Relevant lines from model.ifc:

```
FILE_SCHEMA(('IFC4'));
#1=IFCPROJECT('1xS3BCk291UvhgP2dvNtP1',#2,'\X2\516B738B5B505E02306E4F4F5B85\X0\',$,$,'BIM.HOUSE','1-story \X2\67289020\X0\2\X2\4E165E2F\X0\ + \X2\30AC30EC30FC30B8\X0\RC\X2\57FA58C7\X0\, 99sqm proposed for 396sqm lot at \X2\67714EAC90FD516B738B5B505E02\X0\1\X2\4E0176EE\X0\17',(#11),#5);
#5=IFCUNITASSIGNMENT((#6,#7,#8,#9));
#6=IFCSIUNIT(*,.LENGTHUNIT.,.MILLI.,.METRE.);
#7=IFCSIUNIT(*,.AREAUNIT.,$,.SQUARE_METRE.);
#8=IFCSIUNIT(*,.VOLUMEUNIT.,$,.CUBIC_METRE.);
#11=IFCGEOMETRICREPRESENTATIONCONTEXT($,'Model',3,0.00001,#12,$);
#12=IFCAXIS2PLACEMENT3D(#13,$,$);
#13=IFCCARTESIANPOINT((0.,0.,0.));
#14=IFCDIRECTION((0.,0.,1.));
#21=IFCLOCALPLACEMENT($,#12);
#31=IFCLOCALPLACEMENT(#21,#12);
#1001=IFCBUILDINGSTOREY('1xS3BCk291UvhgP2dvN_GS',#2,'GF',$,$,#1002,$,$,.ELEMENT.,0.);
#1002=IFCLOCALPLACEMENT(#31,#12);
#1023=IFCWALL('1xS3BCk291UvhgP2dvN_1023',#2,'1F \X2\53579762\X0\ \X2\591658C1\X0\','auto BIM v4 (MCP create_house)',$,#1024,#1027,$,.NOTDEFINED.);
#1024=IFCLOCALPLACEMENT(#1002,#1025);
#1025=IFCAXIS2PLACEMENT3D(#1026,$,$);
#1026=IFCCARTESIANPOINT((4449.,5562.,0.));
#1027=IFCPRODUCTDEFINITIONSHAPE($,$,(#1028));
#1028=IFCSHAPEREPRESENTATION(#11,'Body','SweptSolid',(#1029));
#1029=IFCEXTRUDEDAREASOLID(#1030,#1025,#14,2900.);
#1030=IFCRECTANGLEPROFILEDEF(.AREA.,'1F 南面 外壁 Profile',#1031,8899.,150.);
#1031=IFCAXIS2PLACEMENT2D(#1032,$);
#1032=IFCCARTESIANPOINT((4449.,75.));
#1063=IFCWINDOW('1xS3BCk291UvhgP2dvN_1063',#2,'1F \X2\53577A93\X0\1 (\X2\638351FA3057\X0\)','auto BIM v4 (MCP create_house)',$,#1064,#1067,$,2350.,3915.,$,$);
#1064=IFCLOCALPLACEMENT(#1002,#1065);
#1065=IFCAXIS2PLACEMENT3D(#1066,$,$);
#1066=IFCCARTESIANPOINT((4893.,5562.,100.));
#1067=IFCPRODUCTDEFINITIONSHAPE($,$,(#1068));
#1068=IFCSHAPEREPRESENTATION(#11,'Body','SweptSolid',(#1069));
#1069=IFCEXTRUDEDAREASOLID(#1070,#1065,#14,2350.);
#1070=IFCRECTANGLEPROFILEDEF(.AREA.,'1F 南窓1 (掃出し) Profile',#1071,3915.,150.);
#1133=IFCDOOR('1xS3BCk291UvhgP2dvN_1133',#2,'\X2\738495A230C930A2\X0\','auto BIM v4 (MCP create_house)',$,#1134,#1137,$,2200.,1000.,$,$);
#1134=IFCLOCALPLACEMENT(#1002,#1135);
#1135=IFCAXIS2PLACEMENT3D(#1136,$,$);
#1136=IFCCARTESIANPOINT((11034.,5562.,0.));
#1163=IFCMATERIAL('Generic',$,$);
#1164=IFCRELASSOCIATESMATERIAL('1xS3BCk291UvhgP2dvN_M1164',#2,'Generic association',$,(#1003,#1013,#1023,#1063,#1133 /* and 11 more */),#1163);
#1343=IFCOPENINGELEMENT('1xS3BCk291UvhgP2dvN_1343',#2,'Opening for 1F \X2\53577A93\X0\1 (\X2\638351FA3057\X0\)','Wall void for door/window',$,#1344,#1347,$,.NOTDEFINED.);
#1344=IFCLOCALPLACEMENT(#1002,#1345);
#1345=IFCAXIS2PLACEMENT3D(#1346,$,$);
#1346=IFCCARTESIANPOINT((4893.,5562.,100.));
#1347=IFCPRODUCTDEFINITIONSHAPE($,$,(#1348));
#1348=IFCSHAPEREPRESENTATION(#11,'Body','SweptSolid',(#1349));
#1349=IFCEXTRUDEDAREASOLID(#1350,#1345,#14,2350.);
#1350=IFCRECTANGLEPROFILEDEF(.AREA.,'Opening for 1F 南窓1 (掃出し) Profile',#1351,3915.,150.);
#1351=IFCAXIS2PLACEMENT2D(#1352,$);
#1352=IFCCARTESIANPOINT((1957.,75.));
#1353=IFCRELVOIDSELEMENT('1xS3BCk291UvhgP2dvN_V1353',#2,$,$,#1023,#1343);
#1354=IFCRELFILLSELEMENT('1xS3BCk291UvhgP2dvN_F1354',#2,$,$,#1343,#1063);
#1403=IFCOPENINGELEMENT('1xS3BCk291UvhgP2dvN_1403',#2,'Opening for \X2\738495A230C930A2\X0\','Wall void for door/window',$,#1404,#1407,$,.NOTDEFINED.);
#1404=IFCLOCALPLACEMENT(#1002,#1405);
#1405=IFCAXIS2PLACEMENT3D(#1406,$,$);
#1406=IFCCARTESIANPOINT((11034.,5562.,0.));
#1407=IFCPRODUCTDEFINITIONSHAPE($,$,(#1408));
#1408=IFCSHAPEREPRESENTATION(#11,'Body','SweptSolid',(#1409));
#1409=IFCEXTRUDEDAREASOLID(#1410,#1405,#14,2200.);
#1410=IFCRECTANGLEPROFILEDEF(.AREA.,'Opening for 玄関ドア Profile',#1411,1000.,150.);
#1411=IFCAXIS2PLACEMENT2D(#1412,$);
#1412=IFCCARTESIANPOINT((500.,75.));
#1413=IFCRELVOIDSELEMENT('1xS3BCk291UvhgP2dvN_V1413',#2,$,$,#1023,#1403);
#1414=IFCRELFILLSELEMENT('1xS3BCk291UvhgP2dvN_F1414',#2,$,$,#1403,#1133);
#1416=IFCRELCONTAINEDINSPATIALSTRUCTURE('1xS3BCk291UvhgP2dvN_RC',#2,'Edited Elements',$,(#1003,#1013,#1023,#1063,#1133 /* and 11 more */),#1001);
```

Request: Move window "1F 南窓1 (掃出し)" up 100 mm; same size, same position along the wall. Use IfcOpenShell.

```python
import numpy as np
import ifcopenshell
import ifcopenshell.api.geometry
import ifcopenshell.util.placement
import ifcopenshell.util.unit

model = ifcopenshell.open("model.ifc")
unit_scale = ifcopenshell.util.unit.calculate_unit_scale(model)

window = model.by_guid("1xS3BCk291UvhgP2dvN_1063")
opening = window.FillsVoids[0].RelatingOpeningElement
dz = 0.1 / unit_scale

shift = np.array([0.0, 0.0, dz])
# The window is not placed relative to its opening, so move both.
for product in (opening, window):
    matrix = ifcopenshell.util.placement.get_local_placement(product.ObjectPlacement)
    matrix[:3, 3] += shift
    ifcopenshell.api.geometry.edit_object_placement(model, product=product, matrix=matrix, is_si=False)

print(f"moved by {dz * unit_scale:+.3f} m")

model.write("model_v2.ifc")
```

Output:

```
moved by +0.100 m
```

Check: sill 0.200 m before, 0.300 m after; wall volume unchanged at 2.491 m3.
